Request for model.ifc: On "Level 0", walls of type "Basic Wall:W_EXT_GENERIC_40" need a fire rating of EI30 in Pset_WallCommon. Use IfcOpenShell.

First a look at what the model holds.

```python
import ifcopenshell
import ifcopenshell.util.element

model = ifcopenshell.open("model.ifc")
print(model.schema)
storey = next(s for s in model.by_type("IfcBuildingStorey") if s.Name == "Level 0")
walls = [e for e in ifcopenshell.util.element.get_decomposition(storey) if e.is_a("IfcWall")]
seen = {}
for e in walls:
    element_type = ifcopenshell.util.element.get_type(e)
    key = (element_type.Name if element_type != e and element_type else None, ifcopenshell.util.element.get_pset(e, "Pset_WallCommon", "FireRating"))
    seen[key] = seen.get(key, 0) + 1
for (name, value), count in sorted(seen.items(), key=str):
    print(count, "x", name, "|", value)
```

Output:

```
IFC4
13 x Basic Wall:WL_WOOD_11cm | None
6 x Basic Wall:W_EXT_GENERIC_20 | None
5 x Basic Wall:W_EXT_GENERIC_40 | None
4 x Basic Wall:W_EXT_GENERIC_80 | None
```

```python
import ifcopenshell
import ifcopenshell.api.pset
import ifcopenshell.util.element

model = ifcopenshell.open("model.ifc")

storey = next(s for s in model.by_type("IfcBuildingStorey") if s.Name == "Level 0")
walls = [e for e in ifcopenshell.util.element.get_decomposition(storey) if e.is_a("IfcWall")]

count = 0
for e in walls:
    element_type = ifcopenshell.util.element.get_type(e)
    if element_type in (None, e) or element_type.Name != "Basic Wall:W_EXT_GENERIC_40":
        continue
    # add_pset returns the element's existing set when there is one.
    pset = ifcopenshell.api.pset.add_pset(model, product=e, name="Pset_WallCommon")
    ifcopenshell.api.pset.edit_pset(model, pset=pset, properties={"FireRating": "EI30"})
    count += 1

print(count, "walls updated")

model.write("model_edited.ifc")
```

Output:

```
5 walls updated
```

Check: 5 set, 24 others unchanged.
